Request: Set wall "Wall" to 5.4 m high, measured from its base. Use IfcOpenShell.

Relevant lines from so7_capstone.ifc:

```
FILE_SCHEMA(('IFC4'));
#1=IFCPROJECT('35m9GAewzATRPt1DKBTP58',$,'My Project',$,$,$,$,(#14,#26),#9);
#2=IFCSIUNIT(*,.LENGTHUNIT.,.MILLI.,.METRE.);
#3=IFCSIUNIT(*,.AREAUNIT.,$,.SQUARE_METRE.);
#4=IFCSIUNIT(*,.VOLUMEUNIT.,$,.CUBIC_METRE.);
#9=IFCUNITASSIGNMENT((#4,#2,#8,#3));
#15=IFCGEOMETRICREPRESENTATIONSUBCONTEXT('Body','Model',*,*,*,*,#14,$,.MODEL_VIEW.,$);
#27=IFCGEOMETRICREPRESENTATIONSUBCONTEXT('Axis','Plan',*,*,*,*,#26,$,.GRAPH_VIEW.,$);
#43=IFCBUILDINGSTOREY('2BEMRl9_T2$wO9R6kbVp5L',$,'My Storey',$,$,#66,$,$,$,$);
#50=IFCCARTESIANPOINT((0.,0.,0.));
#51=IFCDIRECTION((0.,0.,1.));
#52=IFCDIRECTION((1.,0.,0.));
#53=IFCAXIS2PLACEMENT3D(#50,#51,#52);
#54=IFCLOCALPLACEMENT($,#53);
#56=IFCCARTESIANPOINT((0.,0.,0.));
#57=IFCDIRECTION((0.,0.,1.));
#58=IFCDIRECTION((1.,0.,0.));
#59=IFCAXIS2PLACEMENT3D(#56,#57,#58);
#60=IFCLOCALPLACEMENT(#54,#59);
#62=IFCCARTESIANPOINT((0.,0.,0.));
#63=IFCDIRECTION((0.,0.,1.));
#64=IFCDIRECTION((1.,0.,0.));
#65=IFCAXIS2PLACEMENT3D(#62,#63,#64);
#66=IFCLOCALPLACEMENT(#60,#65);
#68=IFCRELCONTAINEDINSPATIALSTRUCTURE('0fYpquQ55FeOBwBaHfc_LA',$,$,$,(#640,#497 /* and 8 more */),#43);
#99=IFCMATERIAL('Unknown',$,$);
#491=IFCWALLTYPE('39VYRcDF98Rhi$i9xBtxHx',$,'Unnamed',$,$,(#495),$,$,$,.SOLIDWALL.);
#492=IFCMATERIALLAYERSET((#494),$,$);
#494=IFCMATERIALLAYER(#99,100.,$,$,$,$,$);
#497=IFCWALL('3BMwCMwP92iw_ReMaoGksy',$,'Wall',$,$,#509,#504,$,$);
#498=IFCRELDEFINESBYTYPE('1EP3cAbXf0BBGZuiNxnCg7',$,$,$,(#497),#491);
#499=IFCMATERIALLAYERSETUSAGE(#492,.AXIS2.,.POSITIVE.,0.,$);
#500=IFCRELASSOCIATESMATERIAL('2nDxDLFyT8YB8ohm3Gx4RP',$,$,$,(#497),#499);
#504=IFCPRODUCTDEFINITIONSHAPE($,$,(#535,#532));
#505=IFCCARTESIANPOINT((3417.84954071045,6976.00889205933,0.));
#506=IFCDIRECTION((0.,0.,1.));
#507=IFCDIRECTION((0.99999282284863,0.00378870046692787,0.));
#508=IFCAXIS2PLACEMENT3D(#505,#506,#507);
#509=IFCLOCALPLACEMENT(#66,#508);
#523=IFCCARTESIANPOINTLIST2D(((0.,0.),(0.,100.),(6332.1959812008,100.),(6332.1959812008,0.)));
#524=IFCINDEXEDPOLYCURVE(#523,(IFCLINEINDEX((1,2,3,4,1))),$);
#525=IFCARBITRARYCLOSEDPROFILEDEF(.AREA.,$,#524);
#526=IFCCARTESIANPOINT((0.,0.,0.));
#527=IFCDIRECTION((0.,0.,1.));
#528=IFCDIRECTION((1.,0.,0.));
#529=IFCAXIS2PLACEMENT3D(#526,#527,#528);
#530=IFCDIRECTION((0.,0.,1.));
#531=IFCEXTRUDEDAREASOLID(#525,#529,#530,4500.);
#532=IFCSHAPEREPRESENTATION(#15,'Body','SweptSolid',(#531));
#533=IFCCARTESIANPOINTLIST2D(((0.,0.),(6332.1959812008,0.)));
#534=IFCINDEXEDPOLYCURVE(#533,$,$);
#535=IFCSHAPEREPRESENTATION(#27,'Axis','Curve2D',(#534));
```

```python
import ifcopenshell
import ifcopenshell.geom
import ifcopenshell.util.representation
import ifcopenshell.util.shape

model = ifcopenshell.open("so7_capstone.ifc")
settings = ifcopenshell.geom.settings()


def volume(element):
    """Net volume in cubic metres, openings subtracted."""
    shape = ifcopenshell.geom.create_shape(settings, element)
    return ifcopenshell.util.shape.get_volume(shape.geometry)


wall = model.by_guid("3BMwCMwP92iw_ReMaoGksy")
before = volume(wall)

body = ifcopenshell.util.representation.get_representation(wall, "Model", "Body")
solid = body.Items[0]
old_height = solid.Depth
solid.Depth = 5400.0
after = volume(wall)

print(f"height {old_height:g} -> {solid.Depth:g}, volume {before:.3f} -> {after:.3f} m3")

model.write("so7_capstone_v2.ifc")
```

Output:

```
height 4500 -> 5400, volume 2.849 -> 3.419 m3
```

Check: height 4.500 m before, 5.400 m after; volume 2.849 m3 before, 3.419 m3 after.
